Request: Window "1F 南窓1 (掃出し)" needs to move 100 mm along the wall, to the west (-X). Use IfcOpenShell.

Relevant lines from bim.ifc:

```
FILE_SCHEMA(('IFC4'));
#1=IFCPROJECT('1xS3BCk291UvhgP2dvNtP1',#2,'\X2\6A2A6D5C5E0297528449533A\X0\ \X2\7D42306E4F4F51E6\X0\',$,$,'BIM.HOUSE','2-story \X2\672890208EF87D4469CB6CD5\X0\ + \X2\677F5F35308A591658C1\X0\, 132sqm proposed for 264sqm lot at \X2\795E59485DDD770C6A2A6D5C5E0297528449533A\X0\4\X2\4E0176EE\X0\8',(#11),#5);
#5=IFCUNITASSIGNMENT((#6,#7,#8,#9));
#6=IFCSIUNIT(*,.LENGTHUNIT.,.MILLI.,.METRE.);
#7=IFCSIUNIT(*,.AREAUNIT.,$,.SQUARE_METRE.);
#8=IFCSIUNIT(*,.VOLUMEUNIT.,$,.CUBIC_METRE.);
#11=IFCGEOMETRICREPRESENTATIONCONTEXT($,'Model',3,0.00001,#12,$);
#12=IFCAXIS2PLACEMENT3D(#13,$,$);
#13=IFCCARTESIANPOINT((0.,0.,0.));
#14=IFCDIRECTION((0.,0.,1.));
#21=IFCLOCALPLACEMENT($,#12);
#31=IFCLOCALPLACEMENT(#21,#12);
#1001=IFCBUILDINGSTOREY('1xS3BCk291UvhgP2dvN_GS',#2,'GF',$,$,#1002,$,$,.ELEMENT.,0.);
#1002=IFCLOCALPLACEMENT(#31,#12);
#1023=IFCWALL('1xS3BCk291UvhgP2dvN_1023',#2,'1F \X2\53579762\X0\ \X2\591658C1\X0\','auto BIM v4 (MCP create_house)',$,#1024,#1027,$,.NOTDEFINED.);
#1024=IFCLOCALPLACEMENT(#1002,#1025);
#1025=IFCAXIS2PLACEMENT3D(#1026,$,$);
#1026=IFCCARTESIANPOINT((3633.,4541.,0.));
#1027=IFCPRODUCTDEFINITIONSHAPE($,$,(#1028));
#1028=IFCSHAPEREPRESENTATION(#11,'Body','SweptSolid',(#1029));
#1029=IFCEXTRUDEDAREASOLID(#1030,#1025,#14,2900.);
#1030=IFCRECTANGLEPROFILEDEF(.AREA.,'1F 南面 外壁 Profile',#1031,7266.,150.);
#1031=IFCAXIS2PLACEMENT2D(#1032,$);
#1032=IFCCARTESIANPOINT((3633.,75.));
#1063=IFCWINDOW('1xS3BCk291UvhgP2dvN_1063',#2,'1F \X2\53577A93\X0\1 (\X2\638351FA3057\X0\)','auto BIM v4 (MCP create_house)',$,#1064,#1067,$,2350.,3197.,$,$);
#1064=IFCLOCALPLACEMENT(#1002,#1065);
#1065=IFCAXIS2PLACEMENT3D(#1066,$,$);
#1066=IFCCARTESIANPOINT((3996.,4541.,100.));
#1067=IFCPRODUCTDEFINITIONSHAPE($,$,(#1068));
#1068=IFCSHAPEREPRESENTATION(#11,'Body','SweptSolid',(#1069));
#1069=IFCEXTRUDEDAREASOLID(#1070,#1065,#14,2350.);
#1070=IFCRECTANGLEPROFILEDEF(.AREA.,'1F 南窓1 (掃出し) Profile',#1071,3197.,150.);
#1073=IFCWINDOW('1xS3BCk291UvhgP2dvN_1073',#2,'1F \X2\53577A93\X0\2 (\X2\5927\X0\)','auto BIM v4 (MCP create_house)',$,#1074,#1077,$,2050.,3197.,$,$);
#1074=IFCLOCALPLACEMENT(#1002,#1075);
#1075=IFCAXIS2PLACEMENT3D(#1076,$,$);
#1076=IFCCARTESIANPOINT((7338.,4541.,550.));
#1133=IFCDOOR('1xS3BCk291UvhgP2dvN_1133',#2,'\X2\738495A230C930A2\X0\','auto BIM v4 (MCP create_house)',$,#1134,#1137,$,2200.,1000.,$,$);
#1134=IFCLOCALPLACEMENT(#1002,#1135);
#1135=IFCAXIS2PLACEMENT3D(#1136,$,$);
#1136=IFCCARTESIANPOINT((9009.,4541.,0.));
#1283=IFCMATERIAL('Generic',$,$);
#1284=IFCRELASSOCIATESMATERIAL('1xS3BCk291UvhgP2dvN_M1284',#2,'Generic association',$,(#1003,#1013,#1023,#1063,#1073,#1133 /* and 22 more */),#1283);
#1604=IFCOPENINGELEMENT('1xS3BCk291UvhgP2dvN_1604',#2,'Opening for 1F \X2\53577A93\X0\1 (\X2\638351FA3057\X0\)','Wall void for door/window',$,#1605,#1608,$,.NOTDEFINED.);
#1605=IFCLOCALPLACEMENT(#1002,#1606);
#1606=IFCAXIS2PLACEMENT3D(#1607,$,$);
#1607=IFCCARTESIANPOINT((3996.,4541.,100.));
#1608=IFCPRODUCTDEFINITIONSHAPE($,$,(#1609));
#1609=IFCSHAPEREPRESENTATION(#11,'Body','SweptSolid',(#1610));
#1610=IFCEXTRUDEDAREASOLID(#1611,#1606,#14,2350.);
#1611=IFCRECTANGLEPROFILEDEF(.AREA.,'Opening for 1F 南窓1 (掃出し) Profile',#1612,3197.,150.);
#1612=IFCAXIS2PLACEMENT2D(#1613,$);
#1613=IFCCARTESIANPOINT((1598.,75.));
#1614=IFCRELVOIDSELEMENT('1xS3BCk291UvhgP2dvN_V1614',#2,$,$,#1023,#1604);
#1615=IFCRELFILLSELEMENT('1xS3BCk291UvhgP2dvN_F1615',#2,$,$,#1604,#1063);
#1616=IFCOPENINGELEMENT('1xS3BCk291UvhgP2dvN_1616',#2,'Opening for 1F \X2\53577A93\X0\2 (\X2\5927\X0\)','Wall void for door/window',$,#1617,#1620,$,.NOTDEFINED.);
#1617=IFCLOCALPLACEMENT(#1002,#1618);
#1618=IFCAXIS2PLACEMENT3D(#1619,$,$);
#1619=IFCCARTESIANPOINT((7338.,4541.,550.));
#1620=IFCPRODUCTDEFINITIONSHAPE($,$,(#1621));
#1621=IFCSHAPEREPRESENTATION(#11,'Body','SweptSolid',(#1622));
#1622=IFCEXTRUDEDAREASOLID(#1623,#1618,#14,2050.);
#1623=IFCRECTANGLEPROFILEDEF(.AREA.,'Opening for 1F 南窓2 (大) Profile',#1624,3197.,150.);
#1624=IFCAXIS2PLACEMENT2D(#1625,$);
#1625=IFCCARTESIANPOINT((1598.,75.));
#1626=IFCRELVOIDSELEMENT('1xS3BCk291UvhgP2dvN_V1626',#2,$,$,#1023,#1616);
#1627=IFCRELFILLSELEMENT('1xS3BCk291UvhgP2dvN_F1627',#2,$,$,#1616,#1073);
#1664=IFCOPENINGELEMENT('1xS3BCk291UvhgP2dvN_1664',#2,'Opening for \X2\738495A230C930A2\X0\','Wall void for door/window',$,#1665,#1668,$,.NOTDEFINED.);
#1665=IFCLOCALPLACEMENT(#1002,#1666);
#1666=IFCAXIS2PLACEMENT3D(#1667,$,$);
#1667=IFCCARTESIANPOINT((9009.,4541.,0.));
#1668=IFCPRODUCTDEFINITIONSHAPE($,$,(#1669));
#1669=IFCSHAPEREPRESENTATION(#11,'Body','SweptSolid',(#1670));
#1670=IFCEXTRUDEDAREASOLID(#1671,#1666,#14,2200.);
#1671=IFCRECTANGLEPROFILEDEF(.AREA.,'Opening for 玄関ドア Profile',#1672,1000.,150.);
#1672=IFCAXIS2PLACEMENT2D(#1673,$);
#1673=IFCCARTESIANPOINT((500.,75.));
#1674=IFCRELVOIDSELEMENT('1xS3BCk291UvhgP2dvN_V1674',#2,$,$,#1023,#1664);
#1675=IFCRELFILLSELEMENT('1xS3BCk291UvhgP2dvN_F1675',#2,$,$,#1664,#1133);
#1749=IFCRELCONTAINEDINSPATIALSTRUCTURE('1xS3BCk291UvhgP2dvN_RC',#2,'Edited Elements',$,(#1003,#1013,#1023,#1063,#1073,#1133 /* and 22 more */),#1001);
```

```python
import ifcopenshell
import ifcopenshell.api.geometry
import ifcopenshell.util.placement

model = ifcopenshell.open("bim.ifc")

window = model.by_guid("1xS3BCk291UvhgP2dvN_1063")
opening = window.FillsVoids[0].RelatingOpeningElement
wall = opening.VoidsElements[0].RelatingBuildingElement

wall_matrix = ifcopenshell.util.placement.get_local_placement(wall.ObjectPlacement)
shift = wall_matrix[:3, 0] * -100.0
before = ifcopenshell.util.placement.get_local_placement(window.ObjectPlacement)[:3, 3].copy()

# The window is not placed relative to its opening, so move both.
for product in (opening, window):
    matrix = ifcopenshell.util.placement.get_local_placement(product.ObjectPlacement)
    matrix[:3, 3] += shift
    ifcopenshell.api.geometry.edit_object_placement(model, product=product, matrix=matrix, is_si=False)

after = ifcopenshell.util.placement.get_local_placement(window.ObjectPlacement)[:3, 3]
print("window moved by", (after - before).round(3) + 0.0)

model.write("bim_edited.ifc")
```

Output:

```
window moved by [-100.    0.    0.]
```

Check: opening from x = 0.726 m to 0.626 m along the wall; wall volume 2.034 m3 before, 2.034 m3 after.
